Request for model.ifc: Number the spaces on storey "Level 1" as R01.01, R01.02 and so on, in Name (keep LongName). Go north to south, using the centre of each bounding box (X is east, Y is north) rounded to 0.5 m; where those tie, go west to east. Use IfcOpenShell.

First a look at what the model holds.

```python
import ifcopenshell
import ifcopenshell.util.element
import ifcopenshell.util.placement

model = ifcopenshell.open("model.ifc")
print(model.schema)
storey = next(s for s in model.by_type("IfcBuildingStorey") if s.Name == "Level 1")
spaces = [e for e in ifcopenshell.util.element.get_decomposition(storey) if e.is_a("IfcSpace")]
for e in sorted(spaces, key=lambda e: e.id()):
    origin = ifcopenshell.util.placement.get_local_placement(e.ObjectPlacement)[:3, 3]
    print(e.id(), e.Name, e.LongName, origin.round(2) + 0.0, sep=" | ")
```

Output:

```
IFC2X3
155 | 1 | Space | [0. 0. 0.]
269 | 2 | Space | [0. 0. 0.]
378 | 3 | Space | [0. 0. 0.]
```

```python
import ifcopenshell
import ifcopenshell.geom
import ifcopenshell.util.element
import ifcopenshell.util.shape

model = ifcopenshell.open("model.ifc")
settings = ifcopenshell.geom.settings()
settings.set("use-world-coords", True)


def centre(element):
    shape = ifcopenshell.geom.create_shape(settings, element)
    return ifcopenshell.util.shape.get_bbox_centroid(shape.geometry)


storey = next(s for s in model.by_type("IfcBuildingStorey") if s.Name == "Level 1")
spaces = [e for e in ifcopenshell.util.element.get_decomposition(storey) if e.is_a("IfcSpace")]

# Insertion points can sit at a corner or the storey origin, so sort by the geometry (in metres).
centres = {e: centre(e) for e in spaces}
spaces.sort(key=lambda e: (-round(centres[e][1] / 0.5), centres[e][0]))

for i, e in enumerate(spaces, start=1):
    number = f"R01.{i:02d}"
    e.Name = number
    print(e.id(), number)

model.write("model_rev.ifc")
```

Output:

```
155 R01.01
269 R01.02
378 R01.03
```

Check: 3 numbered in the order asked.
